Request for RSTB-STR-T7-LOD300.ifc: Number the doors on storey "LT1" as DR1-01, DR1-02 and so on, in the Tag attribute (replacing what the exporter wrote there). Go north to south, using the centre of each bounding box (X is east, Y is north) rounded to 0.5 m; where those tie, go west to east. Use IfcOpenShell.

First a look at what the model holds.

```python
import ifcopenshell
import ifcopenshell.util.element
import ifcopenshell.util.placement

model = ifcopenshell.open("RSTB-STR-T7-LOD300.ifc")
print(model.schema)
storey = next(s for s in model.by_type("IfcBuildingStorey") if s.Name == "LT1")
doors = [e for e in ifcopenshell.util.element.get_decomposition(storey) if e.is_a("IfcDoor")]
for e in sorted(doors, key=lambda e: e.id()):
    origin = ifcopenshell.util.placement.get_local_placement(e.ObjectPlacement)[:3, 3]
    print(e.id(), e.Tag, e.Name, origin.round(2) + 0.0, sep=" | ")
```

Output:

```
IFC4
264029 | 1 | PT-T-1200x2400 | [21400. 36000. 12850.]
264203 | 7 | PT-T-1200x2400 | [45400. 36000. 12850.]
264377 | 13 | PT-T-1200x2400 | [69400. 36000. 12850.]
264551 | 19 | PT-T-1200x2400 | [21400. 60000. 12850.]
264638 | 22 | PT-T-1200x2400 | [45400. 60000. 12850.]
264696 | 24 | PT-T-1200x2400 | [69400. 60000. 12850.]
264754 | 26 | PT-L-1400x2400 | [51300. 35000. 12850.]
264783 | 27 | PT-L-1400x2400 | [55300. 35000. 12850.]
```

```python
import ifcopenshell
import ifcopenshell.geom
import ifcopenshell.util.element
import ifcopenshell.util.shape

model = ifcopenshell.open("RSTB-STR-T7-LOD300.ifc")
settings = ifcopenshell.geom.settings()
settings.set("use-world-coords", True)


def centre(element):
    shape = ifcopenshell.geom.create_shape(settings, element)
    return ifcopenshell.util.shape.get_bbox_centroid(shape.geometry)


storey = next(s for s in model.by_type("IfcBuildingStorey") if s.Name == "LT1")
doors = [e for e in ifcopenshell.util.element.get_decomposition(storey) if e.is_a("IfcDoor")]

# Insertion points can sit at a corner or the storey origin, so sort by the geometry (in metres).
centres = {e: centre(e) for e in doors}
doors.sort(key=lambda e: (-round(centres[e][1] / 0.5), centres[e][0]))

for i, e in enumerate(doors, start=1):
    number = f"DR1-{i:02d}"
    e.Tag = number
    print(e.id(), number)

model.write("RSTB-STR-T7-LOD300_updated.ifc")
```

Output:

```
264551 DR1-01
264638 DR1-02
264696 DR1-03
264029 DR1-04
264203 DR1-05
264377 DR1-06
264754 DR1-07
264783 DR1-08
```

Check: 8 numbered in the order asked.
